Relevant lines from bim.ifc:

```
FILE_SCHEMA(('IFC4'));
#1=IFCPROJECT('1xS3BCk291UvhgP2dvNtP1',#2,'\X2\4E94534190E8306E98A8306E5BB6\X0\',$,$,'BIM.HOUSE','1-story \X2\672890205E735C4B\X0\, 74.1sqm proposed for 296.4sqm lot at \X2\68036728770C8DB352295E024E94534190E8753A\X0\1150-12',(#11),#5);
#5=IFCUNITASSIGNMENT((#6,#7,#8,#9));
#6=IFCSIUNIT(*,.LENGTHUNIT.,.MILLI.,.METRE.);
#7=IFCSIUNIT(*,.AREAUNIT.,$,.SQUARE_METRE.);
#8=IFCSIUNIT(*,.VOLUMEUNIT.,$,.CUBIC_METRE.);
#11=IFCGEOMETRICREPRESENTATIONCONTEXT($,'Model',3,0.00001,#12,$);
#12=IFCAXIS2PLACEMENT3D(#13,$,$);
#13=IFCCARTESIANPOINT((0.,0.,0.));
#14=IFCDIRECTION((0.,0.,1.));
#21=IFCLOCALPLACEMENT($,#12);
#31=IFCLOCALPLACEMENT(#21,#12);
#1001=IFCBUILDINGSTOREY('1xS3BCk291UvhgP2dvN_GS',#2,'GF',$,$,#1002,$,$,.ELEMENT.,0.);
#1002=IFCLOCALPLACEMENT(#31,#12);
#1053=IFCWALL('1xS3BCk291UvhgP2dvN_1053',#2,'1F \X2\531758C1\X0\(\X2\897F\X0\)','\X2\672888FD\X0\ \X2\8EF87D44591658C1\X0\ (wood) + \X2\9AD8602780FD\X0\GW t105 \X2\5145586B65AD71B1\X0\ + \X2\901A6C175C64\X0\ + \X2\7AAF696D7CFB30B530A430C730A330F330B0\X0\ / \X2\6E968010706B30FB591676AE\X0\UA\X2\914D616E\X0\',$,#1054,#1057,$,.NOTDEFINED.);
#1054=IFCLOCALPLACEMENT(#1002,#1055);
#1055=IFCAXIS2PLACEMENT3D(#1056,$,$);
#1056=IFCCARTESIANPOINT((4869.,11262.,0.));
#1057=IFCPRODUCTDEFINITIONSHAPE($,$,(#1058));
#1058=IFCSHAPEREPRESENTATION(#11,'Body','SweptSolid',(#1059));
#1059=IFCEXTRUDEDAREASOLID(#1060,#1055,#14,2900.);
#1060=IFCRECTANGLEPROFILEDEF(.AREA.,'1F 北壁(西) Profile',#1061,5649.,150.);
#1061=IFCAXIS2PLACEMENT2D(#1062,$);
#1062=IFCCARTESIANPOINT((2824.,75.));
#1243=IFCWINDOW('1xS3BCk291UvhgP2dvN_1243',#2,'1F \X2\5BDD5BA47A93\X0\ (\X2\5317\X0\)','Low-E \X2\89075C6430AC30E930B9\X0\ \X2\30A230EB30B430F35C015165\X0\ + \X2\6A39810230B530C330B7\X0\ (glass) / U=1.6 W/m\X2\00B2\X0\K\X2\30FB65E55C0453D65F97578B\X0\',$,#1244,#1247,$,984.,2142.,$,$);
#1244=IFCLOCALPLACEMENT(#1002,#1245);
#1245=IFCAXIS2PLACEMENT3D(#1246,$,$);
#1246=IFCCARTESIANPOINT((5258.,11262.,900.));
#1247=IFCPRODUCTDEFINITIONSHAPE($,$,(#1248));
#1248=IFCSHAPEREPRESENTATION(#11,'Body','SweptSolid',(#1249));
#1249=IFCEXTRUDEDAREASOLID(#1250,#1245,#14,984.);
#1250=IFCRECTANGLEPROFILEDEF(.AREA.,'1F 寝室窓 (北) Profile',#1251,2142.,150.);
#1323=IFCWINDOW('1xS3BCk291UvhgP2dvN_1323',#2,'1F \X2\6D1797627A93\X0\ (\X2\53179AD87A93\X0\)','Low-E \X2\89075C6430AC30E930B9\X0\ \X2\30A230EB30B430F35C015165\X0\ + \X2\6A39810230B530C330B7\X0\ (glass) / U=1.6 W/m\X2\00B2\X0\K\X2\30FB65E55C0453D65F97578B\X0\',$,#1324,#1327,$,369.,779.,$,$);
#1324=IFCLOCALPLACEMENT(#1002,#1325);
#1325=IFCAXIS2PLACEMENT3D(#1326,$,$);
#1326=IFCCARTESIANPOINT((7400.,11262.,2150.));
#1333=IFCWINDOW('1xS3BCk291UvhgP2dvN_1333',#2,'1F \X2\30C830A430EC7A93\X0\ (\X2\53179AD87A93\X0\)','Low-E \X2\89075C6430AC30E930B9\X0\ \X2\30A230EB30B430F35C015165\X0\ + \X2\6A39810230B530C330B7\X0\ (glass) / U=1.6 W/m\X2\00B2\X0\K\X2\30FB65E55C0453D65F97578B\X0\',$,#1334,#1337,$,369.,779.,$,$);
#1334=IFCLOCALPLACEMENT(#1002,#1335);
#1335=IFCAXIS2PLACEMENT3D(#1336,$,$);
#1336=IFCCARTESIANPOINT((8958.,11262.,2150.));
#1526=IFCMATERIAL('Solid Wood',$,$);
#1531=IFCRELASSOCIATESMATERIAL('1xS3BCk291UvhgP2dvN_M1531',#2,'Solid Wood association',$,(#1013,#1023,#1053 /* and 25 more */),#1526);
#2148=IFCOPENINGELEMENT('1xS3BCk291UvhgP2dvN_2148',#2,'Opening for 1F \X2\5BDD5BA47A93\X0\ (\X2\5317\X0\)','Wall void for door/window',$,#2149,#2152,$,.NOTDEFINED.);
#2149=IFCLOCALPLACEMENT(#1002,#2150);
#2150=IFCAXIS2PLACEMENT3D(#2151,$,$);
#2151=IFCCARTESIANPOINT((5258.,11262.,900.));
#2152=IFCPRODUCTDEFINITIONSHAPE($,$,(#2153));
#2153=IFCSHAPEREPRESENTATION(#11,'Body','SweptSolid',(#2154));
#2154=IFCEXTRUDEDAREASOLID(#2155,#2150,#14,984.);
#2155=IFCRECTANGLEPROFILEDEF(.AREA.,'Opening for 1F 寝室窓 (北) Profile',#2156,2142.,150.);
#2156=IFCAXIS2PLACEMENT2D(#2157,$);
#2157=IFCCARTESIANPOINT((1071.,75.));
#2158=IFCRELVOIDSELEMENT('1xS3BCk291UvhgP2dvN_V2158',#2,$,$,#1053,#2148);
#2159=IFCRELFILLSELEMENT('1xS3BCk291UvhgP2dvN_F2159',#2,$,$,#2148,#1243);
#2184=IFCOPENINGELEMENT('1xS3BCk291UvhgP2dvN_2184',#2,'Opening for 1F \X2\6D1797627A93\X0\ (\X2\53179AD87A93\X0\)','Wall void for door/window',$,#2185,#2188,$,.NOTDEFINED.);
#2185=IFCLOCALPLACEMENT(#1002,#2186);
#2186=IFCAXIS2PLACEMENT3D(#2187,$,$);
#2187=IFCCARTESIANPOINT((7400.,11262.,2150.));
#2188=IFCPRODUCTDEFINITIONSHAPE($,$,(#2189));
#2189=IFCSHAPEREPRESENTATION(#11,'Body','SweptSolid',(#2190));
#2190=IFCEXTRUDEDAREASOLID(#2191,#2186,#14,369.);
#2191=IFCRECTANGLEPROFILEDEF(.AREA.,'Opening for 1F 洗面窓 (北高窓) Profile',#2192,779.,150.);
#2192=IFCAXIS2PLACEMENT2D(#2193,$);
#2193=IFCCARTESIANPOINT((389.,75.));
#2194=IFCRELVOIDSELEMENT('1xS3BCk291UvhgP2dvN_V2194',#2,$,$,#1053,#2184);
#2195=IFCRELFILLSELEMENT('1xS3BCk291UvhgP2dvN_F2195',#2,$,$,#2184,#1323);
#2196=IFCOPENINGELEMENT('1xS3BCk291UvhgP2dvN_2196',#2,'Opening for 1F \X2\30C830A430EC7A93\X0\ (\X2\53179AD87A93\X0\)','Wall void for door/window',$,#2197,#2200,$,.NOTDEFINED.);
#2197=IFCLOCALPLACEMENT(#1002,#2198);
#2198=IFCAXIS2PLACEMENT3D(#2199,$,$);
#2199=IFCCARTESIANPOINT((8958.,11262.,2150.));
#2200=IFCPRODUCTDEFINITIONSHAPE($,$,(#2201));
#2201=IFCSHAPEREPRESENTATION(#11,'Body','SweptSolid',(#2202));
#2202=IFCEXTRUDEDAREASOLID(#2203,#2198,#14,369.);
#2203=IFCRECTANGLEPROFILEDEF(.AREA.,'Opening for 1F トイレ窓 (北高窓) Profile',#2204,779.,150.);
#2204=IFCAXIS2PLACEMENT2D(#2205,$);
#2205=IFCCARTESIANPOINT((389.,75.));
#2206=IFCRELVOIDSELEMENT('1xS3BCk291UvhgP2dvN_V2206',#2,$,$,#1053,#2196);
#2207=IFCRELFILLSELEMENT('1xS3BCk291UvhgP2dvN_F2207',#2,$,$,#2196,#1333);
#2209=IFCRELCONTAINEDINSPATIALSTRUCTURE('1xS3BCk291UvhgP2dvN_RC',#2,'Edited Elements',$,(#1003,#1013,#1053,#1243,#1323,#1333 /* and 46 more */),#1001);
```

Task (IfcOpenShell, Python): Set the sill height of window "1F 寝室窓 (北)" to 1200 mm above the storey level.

```python
import numpy as np
import ifcopenshell
import ifcopenshell.api.geometry
import ifcopenshell.geom
import ifcopenshell.util.element
import ifcopenshell.util.placement
import ifcopenshell.util.shape
import ifcopenshell.util.unit

model = ifcopenshell.open("bim.ifc")
unit_scale = ifcopenshell.util.unit.calculate_unit_scale(model)

window = model.by_guid("1xS3BCk291UvhgP2dvN_1243")
opening = window.FillsVoids[0].RelatingOpeningElement
storey = ifcopenshell.util.element.get_container(window, ifc_class="IfcBuildingStorey")
level = ifcopenshell.util.placement.get_local_placement(storey.ObjectPlacement)[2, 3]

# The opening's origin need not be at the sill, so measure its lowest point.
shape = ifcopenshell.geom.create_shape(ifcopenshell.geom.settings(), opening)
bottom = ifcopenshell.util.shape.get_shape_bottom_elevation(shape, shape.geometry) / unit_scale
dz = level + 1.2 / unit_scale - bottom

shift = np.array([0.0, 0.0, dz])
# The window is not placed relative to its opening, so move both.
for product in (opening, window):
    matrix = ifcopenshell.util.placement.get_local_placement(product.ObjectPlacement)
    matrix[:3, 3] += shift
    ifcopenshell.api.geometry.edit_object_placement(model, product=product, matrix=matrix, is_si=False)

print(f"moved by {dz * unit_scale:+.3f} m")

model.write("bim_updated.ifc")
```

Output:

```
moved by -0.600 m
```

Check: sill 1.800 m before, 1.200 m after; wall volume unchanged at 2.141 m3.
